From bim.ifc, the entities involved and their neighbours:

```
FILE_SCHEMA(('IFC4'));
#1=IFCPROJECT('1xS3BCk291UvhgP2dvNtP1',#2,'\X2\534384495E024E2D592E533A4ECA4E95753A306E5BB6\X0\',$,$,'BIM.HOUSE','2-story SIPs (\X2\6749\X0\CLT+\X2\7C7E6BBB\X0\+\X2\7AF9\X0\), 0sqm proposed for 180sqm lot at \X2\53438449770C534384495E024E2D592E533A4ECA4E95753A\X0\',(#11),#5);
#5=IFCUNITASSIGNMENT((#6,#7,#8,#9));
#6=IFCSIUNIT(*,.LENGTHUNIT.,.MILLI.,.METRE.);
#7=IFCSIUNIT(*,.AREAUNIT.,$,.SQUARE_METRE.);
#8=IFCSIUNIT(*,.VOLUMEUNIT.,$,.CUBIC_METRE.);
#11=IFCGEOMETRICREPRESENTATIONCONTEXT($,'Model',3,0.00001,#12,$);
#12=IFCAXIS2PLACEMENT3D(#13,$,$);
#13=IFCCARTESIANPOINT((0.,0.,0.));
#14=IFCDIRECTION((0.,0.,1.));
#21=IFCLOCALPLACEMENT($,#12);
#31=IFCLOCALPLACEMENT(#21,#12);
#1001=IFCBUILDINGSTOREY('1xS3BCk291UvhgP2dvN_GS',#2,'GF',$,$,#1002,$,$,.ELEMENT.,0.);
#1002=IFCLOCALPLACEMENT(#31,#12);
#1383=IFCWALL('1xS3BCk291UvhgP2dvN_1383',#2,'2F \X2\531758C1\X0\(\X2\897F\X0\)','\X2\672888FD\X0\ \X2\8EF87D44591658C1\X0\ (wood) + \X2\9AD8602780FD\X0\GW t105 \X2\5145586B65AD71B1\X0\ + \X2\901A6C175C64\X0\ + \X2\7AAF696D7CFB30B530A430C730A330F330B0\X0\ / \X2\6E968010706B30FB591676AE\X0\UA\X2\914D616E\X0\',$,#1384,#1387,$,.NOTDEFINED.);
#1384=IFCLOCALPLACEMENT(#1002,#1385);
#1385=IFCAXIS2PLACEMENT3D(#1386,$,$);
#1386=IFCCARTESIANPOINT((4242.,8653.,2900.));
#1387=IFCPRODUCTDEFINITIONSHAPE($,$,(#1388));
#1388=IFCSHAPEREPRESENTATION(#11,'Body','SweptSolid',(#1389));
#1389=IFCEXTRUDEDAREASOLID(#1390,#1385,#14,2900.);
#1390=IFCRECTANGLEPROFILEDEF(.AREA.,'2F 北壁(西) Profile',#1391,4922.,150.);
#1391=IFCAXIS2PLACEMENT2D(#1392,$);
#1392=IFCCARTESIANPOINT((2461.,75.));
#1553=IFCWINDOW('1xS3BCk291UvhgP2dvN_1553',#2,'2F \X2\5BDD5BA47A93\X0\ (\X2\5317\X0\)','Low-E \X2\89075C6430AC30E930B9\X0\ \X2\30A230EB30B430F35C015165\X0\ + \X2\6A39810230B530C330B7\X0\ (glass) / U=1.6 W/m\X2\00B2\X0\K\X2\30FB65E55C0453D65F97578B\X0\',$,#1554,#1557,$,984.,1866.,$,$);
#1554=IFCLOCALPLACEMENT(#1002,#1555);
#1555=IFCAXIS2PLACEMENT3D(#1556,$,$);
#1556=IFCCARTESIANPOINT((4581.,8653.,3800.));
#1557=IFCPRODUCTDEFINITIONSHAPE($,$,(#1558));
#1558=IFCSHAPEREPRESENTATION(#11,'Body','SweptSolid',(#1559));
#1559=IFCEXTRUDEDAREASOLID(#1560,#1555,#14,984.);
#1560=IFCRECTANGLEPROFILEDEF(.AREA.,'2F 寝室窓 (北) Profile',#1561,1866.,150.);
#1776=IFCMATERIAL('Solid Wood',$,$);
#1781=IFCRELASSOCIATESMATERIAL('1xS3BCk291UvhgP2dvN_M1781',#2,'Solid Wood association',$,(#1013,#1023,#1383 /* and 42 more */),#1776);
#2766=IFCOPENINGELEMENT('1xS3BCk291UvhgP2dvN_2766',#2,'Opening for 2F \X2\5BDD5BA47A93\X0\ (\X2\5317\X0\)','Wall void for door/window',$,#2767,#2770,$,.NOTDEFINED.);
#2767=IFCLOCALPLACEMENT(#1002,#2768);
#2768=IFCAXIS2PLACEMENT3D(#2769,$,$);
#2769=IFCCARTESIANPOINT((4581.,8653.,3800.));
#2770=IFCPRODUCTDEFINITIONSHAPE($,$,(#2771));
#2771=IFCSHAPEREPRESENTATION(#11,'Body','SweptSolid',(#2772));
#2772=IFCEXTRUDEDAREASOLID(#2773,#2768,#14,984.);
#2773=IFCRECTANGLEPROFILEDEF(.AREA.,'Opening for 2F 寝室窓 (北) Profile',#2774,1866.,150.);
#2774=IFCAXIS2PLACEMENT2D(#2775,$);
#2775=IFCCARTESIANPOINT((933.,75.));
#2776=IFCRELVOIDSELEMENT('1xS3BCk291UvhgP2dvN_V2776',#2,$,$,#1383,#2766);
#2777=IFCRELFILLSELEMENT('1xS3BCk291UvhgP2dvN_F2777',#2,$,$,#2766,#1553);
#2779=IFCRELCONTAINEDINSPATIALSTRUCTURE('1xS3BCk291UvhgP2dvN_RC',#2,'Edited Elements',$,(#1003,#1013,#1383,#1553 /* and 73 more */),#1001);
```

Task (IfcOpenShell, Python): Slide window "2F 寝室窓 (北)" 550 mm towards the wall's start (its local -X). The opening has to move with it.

```python
import ifcopenshell
import ifcopenshell.api.geometry
import ifcopenshell.util.placement

model = ifcopenshell.open("bim.ifc")

window = model.by_guid("1xS3BCk291UvhgP2dvN_1553")
opening = window.FillsVoids[0].RelatingOpeningElement
wall = opening.VoidsElements[0].RelatingBuildingElement

wall_matrix = ifcopenshell.util.placement.get_local_placement(wall.ObjectPlacement)
shift = wall_matrix[:3, 0] * -550.0
before = ifcopenshell.util.placement.get_local_placement(window.ObjectPlacement)[:3, 3].copy()

# The window is not placed relative to its opening, so move both.
for product in (opening, window):
    matrix = ifcopenshell.util.placement.get_local_placement(product.ObjectPlacement)
    matrix[:3, 3] += shift
    ifcopenshell.api.geometry.edit_object_placement(model, product=product, matrix=matrix, is_si=False)

after = ifcopenshell.util.placement.get_local_placement(window.ObjectPlacement)[:3, 3]
print("window moved by", (after - before).round(3) + 0.0)

model.write("bim_v2.ifc")
```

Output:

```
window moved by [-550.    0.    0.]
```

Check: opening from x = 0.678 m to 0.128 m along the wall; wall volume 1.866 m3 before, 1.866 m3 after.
